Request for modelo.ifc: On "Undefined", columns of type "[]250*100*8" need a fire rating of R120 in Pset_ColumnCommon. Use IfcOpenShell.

First a look at what the model holds.

```python
import ifcopenshell
import ifcopenshell.util.element

model = ifcopenshell.open("modelo.ifc")
print(model.schema)
storey = next(s for s in model.by_type("IfcBuildingStorey") if s.Name == "Undefined")
columns = [e for e in ifcopenshell.util.element.get_decomposition(storey) if e.is_a("IfcColumn")]
seen = {}
for e in columns:
    element_type = ifcopenshell.util.element.get_type(e)
    key = (element_type.Name if element_type != e and element_type else None, ifcopenshell.util.element.get_pset(e, "Pset_ColumnCommon", "FireRating"))
    seen[key] = seen.get(key, 0) + 1
for (name, value), count in sorted(seen.items(), key=str):
    print(count, "x", name, "|", value)
```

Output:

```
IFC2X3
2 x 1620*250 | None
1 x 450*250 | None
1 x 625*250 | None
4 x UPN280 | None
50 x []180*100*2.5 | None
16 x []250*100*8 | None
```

```python
import ifcopenshell
import ifcopenshell.api.pset
import ifcopenshell.util.element

model = ifcopenshell.open("modelo.ifc")

storey = next(s for s in model.by_type("IfcBuildingStorey") if s.Name == "Undefined")
columns = [e for e in ifcopenshell.util.element.get_decomposition(storey) if e.is_a("IfcColumn")]

count = 0
for e in columns:
    element_type = ifcopenshell.util.element.get_type(e)
    if element_type in (None, e) or element_type.Name != "[]250*100*8":
        continue
    found = ifcopenshell.util.element.get_pset(e, "Pset_ColumnCommon", should_inherit=False)
    if found:
        pset = model.by_id(found["id"])
        if len(ifcopenshell.util.element.get_elements_by_pset(pset)) > 1:
            pset = ifcopenshell.api.pset.unshare_pset(model, products=[e], pset=pset)[0]
    else:
        pset = ifcopenshell.api.pset.add_pset(model, product=e, name="Pset_ColumnCommon")
    ifcopenshell.api.pset.edit_pset(model, pset=pset, properties={"FireRating": "R120"})
    count += 1

print(count, "columns updated")

model.write("modelo_v2.ifc")
```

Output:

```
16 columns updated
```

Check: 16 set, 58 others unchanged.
